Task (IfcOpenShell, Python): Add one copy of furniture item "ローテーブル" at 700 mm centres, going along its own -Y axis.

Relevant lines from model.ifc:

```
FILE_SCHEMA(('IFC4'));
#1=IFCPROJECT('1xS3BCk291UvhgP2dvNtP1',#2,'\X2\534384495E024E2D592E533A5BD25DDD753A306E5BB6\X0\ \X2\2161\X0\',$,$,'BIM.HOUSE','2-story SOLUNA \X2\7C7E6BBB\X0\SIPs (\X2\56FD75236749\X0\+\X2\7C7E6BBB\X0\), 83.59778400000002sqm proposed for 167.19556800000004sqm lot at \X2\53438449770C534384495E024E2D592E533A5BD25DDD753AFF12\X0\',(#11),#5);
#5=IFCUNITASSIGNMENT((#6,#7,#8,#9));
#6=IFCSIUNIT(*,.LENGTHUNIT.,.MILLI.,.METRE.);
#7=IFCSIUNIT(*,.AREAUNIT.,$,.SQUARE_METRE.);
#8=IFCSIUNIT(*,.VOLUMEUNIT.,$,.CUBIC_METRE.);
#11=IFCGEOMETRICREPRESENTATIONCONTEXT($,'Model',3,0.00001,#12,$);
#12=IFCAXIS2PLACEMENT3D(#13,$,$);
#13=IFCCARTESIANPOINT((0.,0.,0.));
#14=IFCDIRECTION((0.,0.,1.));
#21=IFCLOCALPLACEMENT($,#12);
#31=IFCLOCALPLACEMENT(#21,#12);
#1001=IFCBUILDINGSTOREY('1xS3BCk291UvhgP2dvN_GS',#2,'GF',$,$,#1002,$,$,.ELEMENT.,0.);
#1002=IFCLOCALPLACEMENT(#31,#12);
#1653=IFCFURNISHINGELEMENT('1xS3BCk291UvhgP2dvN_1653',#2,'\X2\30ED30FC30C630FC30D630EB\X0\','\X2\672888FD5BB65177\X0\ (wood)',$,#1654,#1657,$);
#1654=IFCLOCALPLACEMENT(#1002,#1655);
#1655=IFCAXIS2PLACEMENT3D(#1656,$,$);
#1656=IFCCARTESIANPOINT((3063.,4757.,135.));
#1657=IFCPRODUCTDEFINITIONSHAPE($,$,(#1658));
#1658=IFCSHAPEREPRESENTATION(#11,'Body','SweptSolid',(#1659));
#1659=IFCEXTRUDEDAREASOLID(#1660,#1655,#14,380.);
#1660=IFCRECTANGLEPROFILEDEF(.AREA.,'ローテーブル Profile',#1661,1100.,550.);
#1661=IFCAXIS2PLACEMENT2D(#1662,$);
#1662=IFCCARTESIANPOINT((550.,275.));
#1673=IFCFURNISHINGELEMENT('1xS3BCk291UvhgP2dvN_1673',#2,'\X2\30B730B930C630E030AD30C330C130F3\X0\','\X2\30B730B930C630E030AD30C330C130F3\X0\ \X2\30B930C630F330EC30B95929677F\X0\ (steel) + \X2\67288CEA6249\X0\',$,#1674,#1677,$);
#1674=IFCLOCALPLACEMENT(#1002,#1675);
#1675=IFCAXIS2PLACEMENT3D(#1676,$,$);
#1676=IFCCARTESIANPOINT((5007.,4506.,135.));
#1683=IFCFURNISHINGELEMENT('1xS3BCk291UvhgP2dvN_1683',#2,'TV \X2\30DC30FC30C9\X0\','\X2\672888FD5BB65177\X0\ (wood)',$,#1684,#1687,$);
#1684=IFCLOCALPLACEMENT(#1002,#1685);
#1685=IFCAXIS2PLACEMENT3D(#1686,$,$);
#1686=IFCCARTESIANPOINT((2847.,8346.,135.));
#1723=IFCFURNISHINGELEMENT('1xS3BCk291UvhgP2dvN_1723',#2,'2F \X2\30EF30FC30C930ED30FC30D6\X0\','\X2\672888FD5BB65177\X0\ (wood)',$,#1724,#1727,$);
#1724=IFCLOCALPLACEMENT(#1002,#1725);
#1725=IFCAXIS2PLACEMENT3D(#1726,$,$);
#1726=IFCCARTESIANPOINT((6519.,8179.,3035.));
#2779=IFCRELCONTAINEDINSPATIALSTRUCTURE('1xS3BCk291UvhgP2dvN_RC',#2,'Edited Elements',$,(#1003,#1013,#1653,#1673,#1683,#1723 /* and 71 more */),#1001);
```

```python
import ifcopenshell
import ifcopenshell.api.geometry
import ifcopenshell.api.root
import ifcopenshell.util.element
import ifcopenshell.util.placement

model = ifcopenshell.open("model.ifc")


def reuse_history(source, copy):
    """copy_class also copies each property set's owner history, people and application; keep the originals."""
    for rel in copy.IsDefinedBy:
        if rel.is_a("IfcRelDefinesByProperties") and (history := rel.RelatingPropertyDefinition.OwnerHistory):
            rel.RelatingPropertyDefinition.OwnerHistory = source.OwnerHistory
            ifcopenshell.util.element.remove_deep2(model, history)


source = model.by_guid("1xS3BCk291UvhgP2dvN_1653")
base = ifcopenshell.util.placement.get_local_placement(source.ObjectPlacement)
step = -base[:3, 1] * 700.0

for i in range(1, 2):
    copy = ifcopenshell.api.root.copy_class(model, product=source)
    copy.Representation = ifcopenshell.util.element.copy_deep(
        model, source.Representation, exclude=["IfcGeometricRepresentationContext", "IfcRepresentationMap"]
    )
    reuse_history(source, copy)
    matrix = base.copy()
    matrix[:3, 3] += i * step
    print("added at", matrix[:3, 3].round(3) + 0.0)
    ifcopenshell.api.geometry.edit_object_placement(model, product=copy, matrix=matrix, is_si=False)

model.write("model-out.ifc")
```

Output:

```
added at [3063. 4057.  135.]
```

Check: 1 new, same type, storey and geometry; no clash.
